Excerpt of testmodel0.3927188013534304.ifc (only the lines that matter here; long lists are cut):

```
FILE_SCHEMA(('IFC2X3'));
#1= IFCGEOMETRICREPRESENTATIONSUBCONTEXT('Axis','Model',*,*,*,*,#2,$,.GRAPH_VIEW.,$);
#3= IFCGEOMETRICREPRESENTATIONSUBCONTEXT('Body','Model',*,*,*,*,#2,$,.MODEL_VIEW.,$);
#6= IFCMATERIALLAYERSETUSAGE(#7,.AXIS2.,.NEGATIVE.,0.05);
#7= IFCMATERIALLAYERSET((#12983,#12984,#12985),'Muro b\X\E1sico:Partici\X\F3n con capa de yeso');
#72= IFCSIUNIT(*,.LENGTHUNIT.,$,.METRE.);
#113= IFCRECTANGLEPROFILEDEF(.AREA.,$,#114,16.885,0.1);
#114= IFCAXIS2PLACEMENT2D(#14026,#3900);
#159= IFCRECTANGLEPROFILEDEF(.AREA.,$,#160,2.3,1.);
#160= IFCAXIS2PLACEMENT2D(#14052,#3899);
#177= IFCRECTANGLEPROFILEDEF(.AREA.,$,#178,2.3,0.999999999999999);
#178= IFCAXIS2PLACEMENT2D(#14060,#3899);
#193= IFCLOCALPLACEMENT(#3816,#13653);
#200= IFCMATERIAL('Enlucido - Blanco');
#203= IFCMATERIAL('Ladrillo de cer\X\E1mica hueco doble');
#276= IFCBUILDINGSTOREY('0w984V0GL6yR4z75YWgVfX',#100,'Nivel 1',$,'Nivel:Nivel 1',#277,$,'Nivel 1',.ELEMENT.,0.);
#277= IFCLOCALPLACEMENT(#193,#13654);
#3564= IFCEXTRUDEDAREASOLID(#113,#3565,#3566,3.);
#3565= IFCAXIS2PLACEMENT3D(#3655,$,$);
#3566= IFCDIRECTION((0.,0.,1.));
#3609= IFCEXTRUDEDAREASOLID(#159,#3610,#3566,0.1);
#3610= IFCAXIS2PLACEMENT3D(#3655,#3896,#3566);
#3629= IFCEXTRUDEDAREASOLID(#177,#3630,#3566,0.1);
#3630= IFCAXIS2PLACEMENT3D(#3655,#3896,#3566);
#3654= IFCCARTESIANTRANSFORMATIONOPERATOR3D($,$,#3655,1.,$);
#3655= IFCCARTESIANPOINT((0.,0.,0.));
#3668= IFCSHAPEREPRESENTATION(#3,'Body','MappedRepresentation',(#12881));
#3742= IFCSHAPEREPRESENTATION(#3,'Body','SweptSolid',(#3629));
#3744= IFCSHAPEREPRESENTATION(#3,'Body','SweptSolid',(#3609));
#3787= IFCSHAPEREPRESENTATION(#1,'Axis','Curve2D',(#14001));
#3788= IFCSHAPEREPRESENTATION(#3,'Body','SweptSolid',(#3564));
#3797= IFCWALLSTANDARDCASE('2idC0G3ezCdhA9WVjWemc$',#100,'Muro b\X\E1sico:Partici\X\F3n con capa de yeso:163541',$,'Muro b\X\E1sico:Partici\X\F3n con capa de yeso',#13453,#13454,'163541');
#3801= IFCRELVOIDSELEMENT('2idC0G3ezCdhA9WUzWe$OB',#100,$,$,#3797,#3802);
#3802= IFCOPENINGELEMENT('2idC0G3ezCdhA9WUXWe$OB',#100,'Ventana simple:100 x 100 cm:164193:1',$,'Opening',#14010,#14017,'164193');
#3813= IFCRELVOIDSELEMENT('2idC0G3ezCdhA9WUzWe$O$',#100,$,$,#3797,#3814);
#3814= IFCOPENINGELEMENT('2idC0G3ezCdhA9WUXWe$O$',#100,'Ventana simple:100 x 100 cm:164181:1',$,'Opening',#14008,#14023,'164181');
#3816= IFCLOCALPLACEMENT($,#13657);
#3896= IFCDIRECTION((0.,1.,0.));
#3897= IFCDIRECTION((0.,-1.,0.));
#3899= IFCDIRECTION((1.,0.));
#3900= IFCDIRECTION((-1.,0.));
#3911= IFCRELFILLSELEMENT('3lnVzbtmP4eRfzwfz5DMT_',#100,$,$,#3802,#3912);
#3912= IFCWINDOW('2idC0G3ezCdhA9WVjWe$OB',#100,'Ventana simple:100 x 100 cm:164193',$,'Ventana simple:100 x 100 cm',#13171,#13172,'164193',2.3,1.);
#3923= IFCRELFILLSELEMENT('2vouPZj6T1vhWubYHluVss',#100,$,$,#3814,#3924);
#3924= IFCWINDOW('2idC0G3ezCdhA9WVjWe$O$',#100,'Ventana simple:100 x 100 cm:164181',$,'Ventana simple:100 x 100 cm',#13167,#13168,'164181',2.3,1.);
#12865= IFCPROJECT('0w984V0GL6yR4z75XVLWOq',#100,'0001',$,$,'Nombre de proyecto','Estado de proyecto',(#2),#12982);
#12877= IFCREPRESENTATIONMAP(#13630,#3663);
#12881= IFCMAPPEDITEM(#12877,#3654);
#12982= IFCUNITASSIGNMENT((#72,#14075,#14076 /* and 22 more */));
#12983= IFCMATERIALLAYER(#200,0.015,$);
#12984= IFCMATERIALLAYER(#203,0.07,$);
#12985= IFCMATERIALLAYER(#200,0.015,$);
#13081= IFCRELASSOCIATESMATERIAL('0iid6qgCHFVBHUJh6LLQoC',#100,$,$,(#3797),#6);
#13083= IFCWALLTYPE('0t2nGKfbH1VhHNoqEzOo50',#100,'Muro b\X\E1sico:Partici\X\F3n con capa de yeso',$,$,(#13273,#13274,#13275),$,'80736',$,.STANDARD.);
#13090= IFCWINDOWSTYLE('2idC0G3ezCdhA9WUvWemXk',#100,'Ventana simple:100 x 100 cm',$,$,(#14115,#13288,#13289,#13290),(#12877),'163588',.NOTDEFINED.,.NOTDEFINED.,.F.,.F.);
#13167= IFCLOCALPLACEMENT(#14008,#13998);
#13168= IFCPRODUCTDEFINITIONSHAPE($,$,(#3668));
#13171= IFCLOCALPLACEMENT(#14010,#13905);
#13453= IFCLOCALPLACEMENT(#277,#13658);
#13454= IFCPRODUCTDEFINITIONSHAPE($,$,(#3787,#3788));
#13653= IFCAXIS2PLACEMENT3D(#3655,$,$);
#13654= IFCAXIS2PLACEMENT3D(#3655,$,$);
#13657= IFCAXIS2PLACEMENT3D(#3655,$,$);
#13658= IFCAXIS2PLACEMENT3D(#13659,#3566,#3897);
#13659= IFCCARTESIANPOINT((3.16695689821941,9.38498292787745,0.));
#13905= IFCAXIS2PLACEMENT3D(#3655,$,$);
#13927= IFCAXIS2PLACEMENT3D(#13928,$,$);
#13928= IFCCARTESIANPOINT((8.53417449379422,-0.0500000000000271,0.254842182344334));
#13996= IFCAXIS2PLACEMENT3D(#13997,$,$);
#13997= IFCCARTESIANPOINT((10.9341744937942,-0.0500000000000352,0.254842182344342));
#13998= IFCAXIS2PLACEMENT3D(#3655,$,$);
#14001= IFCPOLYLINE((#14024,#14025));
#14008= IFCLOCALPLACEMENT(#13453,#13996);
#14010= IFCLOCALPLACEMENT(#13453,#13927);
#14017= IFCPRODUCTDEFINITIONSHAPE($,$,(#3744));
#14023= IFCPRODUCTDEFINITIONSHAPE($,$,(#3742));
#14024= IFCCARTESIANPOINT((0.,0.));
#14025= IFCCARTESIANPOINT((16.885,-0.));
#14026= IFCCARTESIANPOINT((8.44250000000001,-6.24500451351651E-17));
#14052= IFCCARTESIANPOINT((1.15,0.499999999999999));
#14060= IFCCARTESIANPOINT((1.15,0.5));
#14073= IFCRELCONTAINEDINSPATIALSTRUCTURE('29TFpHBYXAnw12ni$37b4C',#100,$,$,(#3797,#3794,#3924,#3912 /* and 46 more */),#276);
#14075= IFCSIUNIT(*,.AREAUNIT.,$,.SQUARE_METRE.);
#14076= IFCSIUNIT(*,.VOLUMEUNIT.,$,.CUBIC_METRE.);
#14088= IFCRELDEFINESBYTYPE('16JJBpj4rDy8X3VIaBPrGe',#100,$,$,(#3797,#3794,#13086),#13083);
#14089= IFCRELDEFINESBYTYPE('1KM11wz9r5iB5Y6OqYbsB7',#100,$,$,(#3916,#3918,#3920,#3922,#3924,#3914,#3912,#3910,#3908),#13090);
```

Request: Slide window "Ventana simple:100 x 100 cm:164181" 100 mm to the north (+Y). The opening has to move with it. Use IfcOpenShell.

```python
import ifcopenshell
import ifcopenshell.api.geometry
import ifcopenshell.util.placement

model = ifcopenshell.open("testmodel0.3927188013534304.ifc")

window = model.by_guid("2idC0G3ezCdhA9WVjWe$O$")
opening = window.FillsVoids[0].RelatingOpeningElement
wall = opening.VoidsElements[0].RelatingBuildingElement

wall_matrix = ifcopenshell.util.placement.get_local_placement(wall.ObjectPlacement)
shift = wall_matrix[:3, 0] * -0.1
before = ifcopenshell.util.placement.get_local_placement(window.ObjectPlacement)[:3, 3].copy()

# The window is placed relative to its opening, so it follows when the opening moves.
matrix = ifcopenshell.util.placement.get_local_placement(opening.ObjectPlacement)
matrix[:3, 3] += shift
ifcopenshell.api.geometry.edit_object_placement(
    model, product=opening, matrix=matrix, is_si=False, should_transform_children=True
)

after = ifcopenshell.util.placement.get_local_placement(window.ObjectPlacement)[:3, 3]
print("window moved by", (after - before).round(3) + 0.0)

model.write("testmodel0.3927188013534304_edited.ifc")
```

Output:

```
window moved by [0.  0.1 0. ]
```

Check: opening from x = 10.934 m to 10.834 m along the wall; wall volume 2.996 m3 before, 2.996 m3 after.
